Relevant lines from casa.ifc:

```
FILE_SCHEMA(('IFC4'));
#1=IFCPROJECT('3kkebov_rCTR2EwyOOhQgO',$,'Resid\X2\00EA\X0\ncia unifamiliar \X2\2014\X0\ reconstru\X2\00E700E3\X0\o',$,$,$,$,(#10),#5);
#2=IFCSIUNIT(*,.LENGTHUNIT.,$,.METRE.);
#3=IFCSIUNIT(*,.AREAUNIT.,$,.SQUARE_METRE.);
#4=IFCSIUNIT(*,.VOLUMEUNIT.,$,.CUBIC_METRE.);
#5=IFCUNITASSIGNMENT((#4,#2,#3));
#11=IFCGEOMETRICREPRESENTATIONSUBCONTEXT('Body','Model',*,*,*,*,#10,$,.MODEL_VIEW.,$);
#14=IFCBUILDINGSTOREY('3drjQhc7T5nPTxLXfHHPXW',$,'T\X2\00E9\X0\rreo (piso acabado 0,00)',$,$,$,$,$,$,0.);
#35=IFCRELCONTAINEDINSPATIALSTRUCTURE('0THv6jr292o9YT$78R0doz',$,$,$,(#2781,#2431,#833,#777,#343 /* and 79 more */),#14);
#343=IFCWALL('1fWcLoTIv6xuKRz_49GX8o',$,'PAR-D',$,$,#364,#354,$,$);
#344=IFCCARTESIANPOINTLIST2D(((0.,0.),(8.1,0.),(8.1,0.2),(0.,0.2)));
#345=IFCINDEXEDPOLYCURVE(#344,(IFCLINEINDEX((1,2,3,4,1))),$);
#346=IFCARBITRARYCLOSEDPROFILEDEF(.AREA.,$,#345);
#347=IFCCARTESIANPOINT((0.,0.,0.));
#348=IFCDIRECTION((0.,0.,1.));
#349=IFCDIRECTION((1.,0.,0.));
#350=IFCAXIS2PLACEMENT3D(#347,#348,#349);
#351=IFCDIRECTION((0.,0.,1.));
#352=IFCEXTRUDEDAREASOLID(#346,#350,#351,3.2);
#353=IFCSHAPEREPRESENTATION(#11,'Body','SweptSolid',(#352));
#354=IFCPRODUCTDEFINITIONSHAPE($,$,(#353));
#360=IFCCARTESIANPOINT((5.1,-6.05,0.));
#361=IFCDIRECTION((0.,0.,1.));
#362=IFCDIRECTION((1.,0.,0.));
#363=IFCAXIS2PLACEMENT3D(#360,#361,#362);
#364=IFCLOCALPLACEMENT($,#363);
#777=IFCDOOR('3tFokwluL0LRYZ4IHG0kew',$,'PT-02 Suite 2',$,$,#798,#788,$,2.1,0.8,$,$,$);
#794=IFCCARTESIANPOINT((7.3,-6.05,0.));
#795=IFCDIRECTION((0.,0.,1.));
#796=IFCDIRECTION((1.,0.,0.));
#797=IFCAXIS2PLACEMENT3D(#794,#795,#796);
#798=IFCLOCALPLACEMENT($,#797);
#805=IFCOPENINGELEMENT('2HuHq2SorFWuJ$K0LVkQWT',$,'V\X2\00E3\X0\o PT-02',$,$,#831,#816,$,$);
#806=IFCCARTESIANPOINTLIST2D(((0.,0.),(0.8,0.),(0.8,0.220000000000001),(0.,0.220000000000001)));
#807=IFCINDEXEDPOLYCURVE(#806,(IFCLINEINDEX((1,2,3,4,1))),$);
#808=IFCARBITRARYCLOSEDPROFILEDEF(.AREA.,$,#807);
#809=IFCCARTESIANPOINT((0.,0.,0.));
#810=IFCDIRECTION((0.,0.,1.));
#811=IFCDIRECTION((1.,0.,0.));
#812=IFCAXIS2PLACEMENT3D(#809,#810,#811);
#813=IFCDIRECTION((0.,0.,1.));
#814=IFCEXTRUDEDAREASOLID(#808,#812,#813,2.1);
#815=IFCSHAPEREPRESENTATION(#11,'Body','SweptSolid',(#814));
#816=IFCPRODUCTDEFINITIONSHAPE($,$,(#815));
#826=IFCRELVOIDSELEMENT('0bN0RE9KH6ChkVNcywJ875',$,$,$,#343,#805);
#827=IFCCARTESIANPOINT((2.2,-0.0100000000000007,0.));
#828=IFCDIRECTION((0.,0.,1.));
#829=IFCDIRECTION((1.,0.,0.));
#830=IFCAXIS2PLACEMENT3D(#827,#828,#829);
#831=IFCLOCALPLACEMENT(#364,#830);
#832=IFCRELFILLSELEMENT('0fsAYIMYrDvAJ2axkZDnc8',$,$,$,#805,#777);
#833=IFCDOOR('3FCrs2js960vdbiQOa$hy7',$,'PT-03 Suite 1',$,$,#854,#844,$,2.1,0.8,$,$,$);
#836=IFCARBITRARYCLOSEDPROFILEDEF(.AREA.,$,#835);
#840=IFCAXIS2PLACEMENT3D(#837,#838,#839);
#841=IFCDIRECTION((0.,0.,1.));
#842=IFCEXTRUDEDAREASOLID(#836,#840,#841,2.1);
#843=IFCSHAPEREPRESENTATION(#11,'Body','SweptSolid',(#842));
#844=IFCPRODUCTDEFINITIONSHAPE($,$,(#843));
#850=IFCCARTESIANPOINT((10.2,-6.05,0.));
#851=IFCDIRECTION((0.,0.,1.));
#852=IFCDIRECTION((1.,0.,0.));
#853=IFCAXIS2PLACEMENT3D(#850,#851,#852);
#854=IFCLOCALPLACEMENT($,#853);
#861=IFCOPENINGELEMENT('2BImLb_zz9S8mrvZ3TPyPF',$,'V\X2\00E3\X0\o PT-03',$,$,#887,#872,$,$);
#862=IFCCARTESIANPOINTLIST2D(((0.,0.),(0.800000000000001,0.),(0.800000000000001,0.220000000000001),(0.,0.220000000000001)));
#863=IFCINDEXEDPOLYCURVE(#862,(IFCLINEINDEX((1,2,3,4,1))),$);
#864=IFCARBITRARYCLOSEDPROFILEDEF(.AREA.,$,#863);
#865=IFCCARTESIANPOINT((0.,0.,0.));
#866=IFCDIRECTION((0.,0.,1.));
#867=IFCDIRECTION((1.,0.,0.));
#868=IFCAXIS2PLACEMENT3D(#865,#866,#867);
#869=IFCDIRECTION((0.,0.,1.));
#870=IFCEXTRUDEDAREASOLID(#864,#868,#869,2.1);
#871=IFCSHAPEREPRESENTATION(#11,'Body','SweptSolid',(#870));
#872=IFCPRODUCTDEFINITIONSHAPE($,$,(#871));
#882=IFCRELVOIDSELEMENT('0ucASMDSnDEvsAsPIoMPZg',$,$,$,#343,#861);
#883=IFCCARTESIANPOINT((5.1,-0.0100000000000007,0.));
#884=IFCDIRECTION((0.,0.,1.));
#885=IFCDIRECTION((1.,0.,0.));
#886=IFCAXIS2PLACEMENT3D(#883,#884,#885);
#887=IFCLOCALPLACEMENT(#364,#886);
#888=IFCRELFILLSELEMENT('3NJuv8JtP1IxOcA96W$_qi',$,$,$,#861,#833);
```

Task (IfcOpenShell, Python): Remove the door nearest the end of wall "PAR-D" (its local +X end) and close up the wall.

```python
import ifcopenshell
import ifcopenshell.api.feature
import ifcopenshell.api.root
import ifcopenshell.geom
import ifcopenshell.util.shape

model = ifcopenshell.open("casa.ifc")
settings = ifcopenshell.geom.settings()


def volume(element):
    """Net volume in cubic metres, openings subtracted."""
    shape = ifcopenshell.geom.create_shape(settings, element)
    return ifcopenshell.util.shape.get_volume(shape.geometry)


door = model.by_guid("3FCrs2js960vdbiQOa$hy7")
opening = door.FillsVoids[0].RelatingOpeningElement
wall = opening.VoidsElements[0].RelatingBuildingElement
before = volume(wall)

ifcopenshell.api.root.remove_product(model, product=door)
ifcopenshell.api.feature.remove_feature(model, feature=opening)

after = volume(wall)

print(f"wall volume {before:.3f} -> {after:.3f} m3")

model.write("casa-out.ifc")
```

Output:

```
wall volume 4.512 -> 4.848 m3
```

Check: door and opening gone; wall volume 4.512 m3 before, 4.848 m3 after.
